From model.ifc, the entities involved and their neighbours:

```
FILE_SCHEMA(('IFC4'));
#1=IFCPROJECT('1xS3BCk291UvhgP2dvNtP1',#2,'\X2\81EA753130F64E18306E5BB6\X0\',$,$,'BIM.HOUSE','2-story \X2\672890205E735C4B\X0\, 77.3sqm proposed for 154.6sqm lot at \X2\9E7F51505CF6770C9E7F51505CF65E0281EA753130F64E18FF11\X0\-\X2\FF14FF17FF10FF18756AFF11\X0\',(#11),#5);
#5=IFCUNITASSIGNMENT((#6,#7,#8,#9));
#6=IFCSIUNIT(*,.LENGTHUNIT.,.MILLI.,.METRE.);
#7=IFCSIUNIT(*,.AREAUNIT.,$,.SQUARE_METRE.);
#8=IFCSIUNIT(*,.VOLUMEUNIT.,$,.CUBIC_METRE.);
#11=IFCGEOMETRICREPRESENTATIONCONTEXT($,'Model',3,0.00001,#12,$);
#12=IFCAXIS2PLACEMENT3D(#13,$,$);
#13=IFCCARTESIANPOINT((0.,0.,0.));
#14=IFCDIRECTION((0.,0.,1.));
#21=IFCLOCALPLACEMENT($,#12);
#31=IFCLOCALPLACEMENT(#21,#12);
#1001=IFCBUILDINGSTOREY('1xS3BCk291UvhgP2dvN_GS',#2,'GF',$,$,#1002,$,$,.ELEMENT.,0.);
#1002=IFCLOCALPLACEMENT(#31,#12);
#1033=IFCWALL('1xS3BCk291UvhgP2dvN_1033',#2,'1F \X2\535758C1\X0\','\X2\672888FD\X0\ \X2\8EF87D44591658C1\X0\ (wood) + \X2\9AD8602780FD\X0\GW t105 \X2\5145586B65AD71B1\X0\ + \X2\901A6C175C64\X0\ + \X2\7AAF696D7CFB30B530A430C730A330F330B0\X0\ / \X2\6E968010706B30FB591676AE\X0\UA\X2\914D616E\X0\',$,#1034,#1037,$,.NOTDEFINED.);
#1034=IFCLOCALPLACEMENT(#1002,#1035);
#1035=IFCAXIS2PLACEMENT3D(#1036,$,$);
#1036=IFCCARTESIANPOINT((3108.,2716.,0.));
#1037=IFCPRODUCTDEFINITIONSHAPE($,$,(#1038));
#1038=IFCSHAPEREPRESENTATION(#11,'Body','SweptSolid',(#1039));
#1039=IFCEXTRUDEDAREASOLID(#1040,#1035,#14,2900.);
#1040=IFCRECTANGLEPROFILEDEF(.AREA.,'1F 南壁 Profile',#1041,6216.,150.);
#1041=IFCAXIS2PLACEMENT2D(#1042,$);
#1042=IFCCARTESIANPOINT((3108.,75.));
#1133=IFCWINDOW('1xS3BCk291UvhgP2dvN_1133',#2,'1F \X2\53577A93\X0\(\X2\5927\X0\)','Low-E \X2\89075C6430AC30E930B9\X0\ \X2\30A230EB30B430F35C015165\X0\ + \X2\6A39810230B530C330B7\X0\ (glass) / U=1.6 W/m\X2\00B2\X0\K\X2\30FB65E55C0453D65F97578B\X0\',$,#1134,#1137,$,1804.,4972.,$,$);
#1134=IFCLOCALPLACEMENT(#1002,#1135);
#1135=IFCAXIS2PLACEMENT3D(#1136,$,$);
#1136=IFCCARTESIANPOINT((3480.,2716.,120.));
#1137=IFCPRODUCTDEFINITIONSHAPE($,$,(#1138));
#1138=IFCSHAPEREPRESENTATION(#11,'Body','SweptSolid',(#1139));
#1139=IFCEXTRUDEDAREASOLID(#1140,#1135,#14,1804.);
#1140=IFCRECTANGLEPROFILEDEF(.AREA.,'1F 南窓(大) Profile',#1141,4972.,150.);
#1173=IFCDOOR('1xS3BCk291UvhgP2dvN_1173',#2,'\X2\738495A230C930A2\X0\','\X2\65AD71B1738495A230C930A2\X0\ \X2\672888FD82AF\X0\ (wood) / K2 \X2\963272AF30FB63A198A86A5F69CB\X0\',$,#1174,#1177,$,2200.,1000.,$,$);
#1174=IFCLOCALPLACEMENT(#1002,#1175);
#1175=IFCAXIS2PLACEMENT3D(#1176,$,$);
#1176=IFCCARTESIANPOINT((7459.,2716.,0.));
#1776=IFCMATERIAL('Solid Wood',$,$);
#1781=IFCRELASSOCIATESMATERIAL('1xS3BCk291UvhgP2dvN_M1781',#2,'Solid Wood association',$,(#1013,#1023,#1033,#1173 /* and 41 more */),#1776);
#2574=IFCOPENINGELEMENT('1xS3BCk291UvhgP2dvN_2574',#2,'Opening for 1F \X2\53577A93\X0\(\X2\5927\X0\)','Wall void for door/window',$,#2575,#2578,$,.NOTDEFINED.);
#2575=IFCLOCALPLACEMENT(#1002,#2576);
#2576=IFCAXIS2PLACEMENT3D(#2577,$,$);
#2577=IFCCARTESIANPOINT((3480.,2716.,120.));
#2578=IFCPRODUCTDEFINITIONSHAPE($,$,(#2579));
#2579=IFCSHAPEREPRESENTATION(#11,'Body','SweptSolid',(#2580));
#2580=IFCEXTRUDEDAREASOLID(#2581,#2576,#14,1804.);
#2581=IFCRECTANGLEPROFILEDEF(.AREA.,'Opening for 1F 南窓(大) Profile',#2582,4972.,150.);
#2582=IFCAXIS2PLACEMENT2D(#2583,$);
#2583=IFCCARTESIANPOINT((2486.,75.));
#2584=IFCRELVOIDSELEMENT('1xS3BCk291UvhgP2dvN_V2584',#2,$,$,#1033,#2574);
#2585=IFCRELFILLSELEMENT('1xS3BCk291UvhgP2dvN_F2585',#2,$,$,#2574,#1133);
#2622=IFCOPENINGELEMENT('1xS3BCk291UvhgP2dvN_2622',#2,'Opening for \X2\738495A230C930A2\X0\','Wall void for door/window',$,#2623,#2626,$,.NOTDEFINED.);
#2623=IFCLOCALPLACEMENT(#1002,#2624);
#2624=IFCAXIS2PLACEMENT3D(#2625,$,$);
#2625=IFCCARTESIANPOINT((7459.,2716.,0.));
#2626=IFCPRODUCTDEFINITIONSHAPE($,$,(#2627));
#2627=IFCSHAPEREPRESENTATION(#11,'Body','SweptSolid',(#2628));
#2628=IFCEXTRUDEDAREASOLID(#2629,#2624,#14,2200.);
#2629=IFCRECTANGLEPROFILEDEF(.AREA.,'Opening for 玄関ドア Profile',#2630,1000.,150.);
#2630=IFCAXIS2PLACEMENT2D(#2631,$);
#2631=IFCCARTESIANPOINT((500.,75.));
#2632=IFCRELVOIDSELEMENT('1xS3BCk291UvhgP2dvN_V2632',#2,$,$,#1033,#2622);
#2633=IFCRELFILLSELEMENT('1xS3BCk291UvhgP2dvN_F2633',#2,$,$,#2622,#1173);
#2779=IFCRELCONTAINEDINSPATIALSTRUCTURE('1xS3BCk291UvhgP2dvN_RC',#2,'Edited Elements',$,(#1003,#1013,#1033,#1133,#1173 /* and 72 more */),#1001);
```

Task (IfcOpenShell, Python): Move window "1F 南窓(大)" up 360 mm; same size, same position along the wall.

```python
import numpy as np
import ifcopenshell
import ifcopenshell.api.geometry
import ifcopenshell.util.placement
import ifcopenshell.util.unit

model = ifcopenshell.open("model.ifc")
unit_scale = ifcopenshell.util.unit.calculate_unit_scale(model)

window = model.by_id(1133)
opening = window.FillsVoids[0].RelatingOpeningElement
dz = 0.36 / unit_scale

shift = np.array([0.0, 0.0, dz])
# The window is not placed relative to its opening, so move both.
for product in (opening, window):
    matrix = ifcopenshell.util.placement.get_local_placement(product.ObjectPlacement)
    matrix[:3, 3] += shift
    ifcopenshell.api.geometry.edit_object_placement(model, product=product, matrix=matrix, is_si=False)

print(f"moved by {dz * unit_scale:+.3f} m")

model.write("model_edited.ifc")
```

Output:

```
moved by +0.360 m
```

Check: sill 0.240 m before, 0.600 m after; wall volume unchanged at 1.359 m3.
